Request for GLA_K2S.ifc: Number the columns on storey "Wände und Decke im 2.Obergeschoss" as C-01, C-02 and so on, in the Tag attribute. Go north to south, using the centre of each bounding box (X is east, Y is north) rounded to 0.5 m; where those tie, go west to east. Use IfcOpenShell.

First a look at what the model holds.

```python
import ifcopenshell
import ifcopenshell.util.element
import ifcopenshell.util.placement

model = ifcopenshell.open("GLA_K2S.ifc")
print(model.schema)
storey = next(s for s in model.by_type("IfcBuildingStorey") if s.Name == "Wände und Decke im 2.Obergeschoss")
columns = [e for e in ifcopenshell.util.element.get_decomposition(storey) if e.is_a("IfcColumn")]
for e in sorted(columns, key=lambda e: e.id()):
    origin = ifcopenshell.util.placement.get_local_placement(e.ObjectPlacement)[:3, 3]
    print(e.id(), e.Tag, e.Name, origin.round(2) + 0.0, sep=" | ")
```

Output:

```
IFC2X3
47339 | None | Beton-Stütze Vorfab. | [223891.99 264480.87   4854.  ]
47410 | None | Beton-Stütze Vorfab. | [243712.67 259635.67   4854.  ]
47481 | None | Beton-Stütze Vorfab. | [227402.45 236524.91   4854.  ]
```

```python
import ifcopenshell
import ifcopenshell.geom
import ifcopenshell.util.element
import ifcopenshell.util.shape

model = ifcopenshell.open("GLA_K2S.ifc")
settings = ifcopenshell.geom.settings()
settings.set("use-world-coords", True)


def centre(element):
    shape = ifcopenshell.geom.create_shape(settings, element)
    return ifcopenshell.util.shape.get_bbox_centroid(shape.geometry)


storey = next(s for s in model.by_type("IfcBuildingStorey") if s.Name == "Wände und Decke im 2.Obergeschoss")
columns = [e for e in ifcopenshell.util.element.get_decomposition(storey) if e.is_a("IfcColumn")]

# Insertion points can sit at a corner or the storey origin, so sort by the geometry (in metres).
centres = {e: centre(e) for e in columns}
columns.sort(key=lambda e: (-round(centres[e][1] / 0.5), centres[e][0]))

for i, e in enumerate(columns, start=1):
    number = f"C-{i:02d}"
    e.Tag = number
    print(e.id(), number)

model.write("GLA_K2S_rev.ifc")
```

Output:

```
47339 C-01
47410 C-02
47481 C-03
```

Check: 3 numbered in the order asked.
